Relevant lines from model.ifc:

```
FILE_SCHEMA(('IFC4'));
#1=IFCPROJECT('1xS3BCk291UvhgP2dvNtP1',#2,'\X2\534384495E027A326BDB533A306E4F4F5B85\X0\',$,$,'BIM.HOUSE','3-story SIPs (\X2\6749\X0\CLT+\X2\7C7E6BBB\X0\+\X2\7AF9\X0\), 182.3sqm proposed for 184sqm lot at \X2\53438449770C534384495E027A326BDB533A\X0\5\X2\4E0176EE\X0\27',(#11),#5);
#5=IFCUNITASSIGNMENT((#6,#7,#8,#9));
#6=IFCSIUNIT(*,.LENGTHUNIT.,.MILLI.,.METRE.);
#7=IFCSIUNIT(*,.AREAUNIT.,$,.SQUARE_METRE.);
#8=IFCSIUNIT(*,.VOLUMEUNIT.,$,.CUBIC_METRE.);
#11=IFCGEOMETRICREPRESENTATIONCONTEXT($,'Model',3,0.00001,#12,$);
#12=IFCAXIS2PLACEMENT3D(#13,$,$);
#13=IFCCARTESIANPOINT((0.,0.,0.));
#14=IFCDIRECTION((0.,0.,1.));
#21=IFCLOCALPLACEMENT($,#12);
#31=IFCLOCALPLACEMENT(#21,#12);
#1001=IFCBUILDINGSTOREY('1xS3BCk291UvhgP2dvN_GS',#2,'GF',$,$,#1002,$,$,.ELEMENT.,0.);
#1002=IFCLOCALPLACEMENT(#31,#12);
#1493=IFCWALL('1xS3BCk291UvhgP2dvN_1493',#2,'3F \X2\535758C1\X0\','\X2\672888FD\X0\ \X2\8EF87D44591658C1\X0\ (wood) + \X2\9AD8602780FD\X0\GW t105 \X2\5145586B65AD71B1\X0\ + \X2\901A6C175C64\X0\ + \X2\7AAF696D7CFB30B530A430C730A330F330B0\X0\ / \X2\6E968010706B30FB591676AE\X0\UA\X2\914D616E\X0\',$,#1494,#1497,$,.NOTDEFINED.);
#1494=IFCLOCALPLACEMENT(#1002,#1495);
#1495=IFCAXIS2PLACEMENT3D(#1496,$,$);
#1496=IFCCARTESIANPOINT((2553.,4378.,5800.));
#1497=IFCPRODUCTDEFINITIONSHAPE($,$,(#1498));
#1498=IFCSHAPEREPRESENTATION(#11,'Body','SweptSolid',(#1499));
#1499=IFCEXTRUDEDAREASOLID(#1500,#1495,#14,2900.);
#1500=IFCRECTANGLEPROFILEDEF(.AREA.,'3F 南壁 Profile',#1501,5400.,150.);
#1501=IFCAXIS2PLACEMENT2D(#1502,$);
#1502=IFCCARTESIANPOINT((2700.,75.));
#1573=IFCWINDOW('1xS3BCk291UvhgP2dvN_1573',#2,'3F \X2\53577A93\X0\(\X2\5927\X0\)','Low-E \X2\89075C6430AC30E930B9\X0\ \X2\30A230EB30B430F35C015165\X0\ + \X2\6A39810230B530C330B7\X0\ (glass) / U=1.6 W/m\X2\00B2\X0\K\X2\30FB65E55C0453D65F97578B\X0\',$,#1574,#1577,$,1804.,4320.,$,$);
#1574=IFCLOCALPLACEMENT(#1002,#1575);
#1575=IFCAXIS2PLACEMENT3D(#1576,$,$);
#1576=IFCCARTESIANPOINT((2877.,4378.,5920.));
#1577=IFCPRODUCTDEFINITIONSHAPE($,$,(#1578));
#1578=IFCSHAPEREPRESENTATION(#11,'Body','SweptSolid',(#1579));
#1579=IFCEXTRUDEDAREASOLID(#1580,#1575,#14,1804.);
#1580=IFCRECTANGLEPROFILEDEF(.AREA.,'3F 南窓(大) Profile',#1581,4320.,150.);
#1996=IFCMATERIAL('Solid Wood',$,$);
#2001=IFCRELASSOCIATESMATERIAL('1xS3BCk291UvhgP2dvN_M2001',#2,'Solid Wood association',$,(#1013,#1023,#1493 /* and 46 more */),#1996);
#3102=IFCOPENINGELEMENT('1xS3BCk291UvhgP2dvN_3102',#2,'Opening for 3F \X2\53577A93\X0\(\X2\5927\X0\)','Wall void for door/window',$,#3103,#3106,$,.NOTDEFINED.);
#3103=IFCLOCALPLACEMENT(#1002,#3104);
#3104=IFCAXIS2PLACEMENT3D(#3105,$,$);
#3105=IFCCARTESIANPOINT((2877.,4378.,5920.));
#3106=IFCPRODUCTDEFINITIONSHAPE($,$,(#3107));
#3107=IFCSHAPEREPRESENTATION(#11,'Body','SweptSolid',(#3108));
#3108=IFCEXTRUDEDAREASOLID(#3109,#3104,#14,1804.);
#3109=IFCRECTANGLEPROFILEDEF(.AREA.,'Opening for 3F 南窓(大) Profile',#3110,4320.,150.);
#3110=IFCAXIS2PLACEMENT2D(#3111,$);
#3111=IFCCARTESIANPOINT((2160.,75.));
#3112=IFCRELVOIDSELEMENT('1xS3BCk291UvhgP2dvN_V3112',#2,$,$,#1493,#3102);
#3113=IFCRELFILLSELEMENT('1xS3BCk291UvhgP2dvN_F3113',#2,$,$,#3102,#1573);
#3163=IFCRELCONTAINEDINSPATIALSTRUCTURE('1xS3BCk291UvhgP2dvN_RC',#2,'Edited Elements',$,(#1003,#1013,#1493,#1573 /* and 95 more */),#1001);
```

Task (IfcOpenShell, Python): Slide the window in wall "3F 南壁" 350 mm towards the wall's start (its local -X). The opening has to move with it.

```python
import ifcopenshell
import ifcopenshell.api.geometry
import ifcopenshell.util.placement
import ifcopenshell.util.unit

model = ifcopenshell.open("model.ifc")
unit_scale = ifcopenshell.util.unit.calculate_unit_scale(model)

window = model.by_id(1573)
opening = window.FillsVoids[0].RelatingOpeningElement
wall = opening.VoidsElements[0].RelatingBuildingElement

wall_matrix = ifcopenshell.util.placement.get_local_placement(wall.ObjectPlacement)
shift = wall_matrix[:3, 0] * -0.35 / unit_scale
before = ifcopenshell.util.placement.get_local_placement(window.ObjectPlacement)[:3, 3].copy()

# The window is not placed relative to its opening, so move both.
for product in (opening, window):
    matrix = ifcopenshell.util.placement.get_local_placement(product.ObjectPlacement)
    matrix[:3, 3] += shift
    ifcopenshell.api.geometry.edit_object_placement(model, product=product, matrix=matrix, is_si=False)

after = ifcopenshell.util.placement.get_local_placement(window.ObjectPlacement)[:3, 3]
print("window moved by", (after - before).round(3) + 0.0)

model.write("model_rev.ifc")
```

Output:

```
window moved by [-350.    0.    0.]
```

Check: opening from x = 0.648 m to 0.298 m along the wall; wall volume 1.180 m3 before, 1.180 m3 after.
